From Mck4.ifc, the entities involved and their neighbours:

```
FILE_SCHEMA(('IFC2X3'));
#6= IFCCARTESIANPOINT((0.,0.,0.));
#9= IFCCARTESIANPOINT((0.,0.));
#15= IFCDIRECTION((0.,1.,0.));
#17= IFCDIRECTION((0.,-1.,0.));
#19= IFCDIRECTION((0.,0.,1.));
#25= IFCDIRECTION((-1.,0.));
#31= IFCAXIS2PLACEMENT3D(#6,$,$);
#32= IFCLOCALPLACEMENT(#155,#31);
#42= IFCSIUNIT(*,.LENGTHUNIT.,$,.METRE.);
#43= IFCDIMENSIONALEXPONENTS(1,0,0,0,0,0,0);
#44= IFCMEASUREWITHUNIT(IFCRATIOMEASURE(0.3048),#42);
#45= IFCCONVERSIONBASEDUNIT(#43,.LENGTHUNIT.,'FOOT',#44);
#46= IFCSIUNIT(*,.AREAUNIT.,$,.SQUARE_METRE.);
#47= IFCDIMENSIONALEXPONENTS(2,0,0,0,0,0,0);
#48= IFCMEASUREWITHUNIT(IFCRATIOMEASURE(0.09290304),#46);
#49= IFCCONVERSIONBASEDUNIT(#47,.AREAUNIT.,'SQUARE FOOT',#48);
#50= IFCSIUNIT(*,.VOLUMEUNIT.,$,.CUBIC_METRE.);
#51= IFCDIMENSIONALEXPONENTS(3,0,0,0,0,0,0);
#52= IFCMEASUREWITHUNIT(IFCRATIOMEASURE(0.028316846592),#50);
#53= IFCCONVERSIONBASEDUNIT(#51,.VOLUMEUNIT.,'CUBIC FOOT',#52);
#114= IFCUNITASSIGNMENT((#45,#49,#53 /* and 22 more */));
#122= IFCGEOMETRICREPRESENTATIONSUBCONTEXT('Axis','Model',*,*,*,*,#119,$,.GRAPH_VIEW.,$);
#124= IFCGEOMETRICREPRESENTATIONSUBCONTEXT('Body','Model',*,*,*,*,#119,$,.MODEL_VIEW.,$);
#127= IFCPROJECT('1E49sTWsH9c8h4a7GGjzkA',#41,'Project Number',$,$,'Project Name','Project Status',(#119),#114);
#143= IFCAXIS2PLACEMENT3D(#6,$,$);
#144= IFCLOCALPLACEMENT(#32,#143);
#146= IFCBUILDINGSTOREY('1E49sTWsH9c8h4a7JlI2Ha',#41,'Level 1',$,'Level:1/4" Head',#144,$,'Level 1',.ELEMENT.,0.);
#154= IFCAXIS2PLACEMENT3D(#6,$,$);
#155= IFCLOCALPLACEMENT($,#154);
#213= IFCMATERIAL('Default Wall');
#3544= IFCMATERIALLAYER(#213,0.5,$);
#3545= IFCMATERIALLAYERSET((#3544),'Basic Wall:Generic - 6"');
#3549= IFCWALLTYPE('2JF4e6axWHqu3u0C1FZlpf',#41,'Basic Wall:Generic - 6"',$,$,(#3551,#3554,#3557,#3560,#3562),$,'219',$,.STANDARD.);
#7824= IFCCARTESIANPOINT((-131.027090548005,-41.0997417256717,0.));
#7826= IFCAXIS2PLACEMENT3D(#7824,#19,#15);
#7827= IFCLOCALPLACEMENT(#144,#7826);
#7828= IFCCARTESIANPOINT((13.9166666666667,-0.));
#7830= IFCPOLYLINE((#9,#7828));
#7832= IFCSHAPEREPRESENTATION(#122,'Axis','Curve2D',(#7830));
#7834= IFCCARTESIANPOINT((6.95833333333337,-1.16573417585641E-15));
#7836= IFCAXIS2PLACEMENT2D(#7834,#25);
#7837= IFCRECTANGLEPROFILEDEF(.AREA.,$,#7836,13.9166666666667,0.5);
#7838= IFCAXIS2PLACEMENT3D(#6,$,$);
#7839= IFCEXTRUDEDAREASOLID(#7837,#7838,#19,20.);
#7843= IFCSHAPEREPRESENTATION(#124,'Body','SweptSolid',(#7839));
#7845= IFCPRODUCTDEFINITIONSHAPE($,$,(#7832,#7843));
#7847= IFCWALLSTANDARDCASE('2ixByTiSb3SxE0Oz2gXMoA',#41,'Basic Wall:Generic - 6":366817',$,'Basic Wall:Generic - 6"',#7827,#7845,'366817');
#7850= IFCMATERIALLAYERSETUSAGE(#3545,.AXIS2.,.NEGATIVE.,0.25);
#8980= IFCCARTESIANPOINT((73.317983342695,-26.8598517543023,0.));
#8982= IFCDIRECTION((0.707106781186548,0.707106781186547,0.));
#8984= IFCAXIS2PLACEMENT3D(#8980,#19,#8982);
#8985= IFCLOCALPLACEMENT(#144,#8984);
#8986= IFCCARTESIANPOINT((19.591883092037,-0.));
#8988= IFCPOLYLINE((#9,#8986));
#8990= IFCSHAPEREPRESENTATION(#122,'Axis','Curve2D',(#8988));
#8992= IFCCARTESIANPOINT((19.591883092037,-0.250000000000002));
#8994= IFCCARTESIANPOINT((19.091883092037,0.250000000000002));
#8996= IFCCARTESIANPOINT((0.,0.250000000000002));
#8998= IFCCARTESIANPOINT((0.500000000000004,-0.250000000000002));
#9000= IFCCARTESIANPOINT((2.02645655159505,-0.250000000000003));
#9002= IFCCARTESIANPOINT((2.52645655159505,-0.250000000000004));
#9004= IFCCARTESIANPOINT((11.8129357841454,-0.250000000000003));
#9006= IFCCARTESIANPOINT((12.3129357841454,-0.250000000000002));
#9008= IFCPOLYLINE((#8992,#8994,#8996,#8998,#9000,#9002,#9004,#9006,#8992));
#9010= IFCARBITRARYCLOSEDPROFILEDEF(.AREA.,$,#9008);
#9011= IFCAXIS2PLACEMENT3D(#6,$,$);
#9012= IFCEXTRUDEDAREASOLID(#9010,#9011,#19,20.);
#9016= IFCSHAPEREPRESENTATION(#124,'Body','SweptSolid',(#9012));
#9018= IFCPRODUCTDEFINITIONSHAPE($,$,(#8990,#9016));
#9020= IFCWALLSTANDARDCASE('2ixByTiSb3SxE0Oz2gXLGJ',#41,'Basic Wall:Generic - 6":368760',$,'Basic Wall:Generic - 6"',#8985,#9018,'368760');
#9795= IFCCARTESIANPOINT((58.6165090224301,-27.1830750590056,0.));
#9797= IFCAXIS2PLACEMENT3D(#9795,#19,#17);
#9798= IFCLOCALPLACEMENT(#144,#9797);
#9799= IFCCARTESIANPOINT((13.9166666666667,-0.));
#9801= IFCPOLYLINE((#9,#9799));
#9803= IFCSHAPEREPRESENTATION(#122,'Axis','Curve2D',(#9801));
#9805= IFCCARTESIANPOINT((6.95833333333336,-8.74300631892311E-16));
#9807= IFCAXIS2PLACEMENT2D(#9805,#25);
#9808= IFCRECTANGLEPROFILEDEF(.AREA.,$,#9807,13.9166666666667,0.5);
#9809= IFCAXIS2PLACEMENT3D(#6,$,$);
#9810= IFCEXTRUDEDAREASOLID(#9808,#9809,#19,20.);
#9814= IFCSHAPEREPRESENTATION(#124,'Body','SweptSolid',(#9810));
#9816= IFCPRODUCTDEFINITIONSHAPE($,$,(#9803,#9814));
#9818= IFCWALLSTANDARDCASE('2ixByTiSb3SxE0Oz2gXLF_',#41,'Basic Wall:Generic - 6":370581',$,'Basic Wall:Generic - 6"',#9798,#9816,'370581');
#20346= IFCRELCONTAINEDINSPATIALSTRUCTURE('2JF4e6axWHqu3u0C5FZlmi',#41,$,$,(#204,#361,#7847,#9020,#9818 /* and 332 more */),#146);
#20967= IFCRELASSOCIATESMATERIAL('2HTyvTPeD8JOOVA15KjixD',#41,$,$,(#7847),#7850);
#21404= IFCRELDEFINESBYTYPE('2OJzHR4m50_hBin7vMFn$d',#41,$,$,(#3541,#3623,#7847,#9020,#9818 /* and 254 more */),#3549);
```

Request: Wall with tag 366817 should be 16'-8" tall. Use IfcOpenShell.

```python
import ifcopenshell
import ifcopenshell.geom
import ifcopenshell.util.representation
import ifcopenshell.util.shape
import ifcopenshell.util.unit

model = ifcopenshell.open("Mck4.ifc")
unit_scale = ifcopenshell.util.unit.calculate_unit_scale(model)
settings = ifcopenshell.geom.settings()


def volume(element):
    """Net volume in cubic metres, openings subtracted."""
    shape = ifcopenshell.geom.create_shape(settings, element)
    return ifcopenshell.util.shape.get_volume(shape.geometry)


wall = model.by_id(7847)
before = volume(wall)

body = ifcopenshell.util.representation.get_representation(wall, "Model", "Body")
solid = body.Items[0]
old_height = solid.Depth
solid.Depth = 200 * 0.0254 / unit_scale
after = volume(wall)

print(f"height {old_height:g} -> {solid.Depth:g}, volume {before:.3f} -> {after:.3f} m3")

model.write("Mck4-out.ifc")
```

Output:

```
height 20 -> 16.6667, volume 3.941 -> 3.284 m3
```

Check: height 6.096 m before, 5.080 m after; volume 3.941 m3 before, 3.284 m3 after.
